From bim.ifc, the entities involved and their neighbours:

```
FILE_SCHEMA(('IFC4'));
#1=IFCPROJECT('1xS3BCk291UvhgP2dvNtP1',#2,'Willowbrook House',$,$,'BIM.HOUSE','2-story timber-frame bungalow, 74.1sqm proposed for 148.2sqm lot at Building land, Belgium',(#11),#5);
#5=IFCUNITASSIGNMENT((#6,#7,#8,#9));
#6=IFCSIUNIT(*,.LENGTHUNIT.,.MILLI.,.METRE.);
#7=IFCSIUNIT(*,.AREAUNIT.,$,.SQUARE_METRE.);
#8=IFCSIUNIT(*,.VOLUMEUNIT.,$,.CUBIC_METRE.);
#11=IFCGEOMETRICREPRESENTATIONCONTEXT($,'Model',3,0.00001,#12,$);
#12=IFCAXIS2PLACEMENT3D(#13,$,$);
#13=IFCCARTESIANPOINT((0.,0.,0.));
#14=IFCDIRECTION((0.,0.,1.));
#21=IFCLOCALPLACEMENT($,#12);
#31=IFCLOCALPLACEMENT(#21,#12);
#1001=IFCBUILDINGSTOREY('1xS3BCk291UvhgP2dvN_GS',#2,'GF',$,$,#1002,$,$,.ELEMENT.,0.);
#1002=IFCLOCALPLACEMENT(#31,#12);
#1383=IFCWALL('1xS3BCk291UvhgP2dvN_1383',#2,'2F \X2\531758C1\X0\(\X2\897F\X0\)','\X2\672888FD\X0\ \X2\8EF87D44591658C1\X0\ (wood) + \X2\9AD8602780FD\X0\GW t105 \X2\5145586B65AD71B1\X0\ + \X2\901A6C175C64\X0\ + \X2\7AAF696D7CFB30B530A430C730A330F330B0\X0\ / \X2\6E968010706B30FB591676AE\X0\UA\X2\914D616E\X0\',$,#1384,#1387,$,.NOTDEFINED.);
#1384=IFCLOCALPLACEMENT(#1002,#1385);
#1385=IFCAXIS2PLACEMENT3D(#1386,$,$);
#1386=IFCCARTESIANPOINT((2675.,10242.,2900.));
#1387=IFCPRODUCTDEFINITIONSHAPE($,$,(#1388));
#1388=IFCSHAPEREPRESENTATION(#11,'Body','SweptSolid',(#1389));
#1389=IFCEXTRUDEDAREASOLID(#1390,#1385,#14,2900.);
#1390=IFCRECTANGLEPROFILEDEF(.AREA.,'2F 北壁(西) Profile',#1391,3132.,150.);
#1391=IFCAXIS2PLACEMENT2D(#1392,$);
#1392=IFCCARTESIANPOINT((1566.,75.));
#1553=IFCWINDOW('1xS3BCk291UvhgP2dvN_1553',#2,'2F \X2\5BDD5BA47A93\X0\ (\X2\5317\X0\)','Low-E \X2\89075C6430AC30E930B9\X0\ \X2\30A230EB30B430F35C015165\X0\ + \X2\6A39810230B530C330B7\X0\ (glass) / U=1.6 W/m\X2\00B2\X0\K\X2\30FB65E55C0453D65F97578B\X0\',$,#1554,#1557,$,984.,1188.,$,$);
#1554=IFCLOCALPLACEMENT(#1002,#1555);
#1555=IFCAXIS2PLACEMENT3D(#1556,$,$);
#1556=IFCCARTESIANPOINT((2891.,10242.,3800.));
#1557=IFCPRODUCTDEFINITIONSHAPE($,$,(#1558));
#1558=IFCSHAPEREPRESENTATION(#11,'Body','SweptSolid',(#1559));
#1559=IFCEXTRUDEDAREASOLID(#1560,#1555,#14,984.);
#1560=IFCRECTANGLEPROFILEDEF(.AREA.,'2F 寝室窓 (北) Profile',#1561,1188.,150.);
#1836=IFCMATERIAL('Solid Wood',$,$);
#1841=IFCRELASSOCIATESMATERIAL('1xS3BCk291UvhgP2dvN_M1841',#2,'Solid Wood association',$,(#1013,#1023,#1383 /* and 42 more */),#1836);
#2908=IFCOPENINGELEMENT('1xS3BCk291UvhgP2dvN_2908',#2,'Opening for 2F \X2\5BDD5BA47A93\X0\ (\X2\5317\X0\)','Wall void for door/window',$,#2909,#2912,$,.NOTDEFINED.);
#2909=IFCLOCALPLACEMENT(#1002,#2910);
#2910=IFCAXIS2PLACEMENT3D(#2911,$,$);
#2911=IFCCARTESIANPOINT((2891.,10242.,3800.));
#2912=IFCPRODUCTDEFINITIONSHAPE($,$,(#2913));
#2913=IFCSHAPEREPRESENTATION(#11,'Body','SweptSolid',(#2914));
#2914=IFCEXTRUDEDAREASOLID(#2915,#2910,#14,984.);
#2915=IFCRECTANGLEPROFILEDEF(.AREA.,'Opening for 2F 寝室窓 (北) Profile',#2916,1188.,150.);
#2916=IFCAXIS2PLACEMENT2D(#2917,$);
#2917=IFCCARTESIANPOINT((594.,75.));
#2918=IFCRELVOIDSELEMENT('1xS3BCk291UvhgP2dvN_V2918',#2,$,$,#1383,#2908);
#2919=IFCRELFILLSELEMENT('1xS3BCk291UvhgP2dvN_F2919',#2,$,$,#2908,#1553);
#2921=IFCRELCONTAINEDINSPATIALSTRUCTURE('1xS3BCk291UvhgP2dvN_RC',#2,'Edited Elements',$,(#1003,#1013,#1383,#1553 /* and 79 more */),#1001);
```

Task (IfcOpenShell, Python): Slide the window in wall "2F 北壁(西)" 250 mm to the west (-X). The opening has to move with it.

```python
import ifcopenshell
import ifcopenshell.api.geometry
import ifcopenshell.util.placement
import ifcopenshell.util.unit

model = ifcopenshell.open("bim.ifc")
unit_scale = ifcopenshell.util.unit.calculate_unit_scale(model)

window = model.by_guid("1xS3BCk291UvhgP2dvN_1553")
opening = window.FillsVoids[0].RelatingOpeningElement
wall = opening.VoidsElements[0].RelatingBuildingElement

wall_matrix = ifcopenshell.util.placement.get_local_placement(wall.ObjectPlacement)
shift = wall_matrix[:3, 0] * -0.25 / unit_scale
before = ifcopenshell.util.placement.get_local_placement(window.ObjectPlacement)[:3, 3].copy()

# The window is not placed relative to its opening, so move both.
for product in (opening, window):
    matrix = ifcopenshell.util.placement.get_local_placement(product.ObjectPlacement)
    matrix[:3, 3] += shift
    ifcopenshell.api.geometry.edit_object_placement(model, product=product, matrix=matrix, is_si=False)

after = ifcopenshell.util.placement.get_local_placement(window.ObjectPlacement)[:3, 3]
print("window moved by", (after - before).round(3) + 0.0)

model.write("bim_rev.ifc")
```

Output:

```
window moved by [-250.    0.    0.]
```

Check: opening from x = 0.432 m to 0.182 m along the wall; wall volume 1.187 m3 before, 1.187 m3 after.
